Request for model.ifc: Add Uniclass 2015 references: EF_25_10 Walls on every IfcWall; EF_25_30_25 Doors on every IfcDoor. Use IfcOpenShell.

First a look at what the model holds.

```python
import ifcopenshell

model = ifcopenshell.open("model.ifc")
print(model.schema)
print("classifications:", [c.Name for c in model.by_type("IfcClassification")])
for ifc_class in ("IfcDoor", "IfcRoof", "IfcStair", "IfcWall", "IfcWindow"):
    print(ifc_class, len(model.by_type(ifc_class)))
```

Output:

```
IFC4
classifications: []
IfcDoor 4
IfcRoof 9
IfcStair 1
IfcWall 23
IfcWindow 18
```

```python
import ifcopenshell
import ifcopenshell.api.classification

model = ifcopenshell.open("model.ifc")

system = ifcopenshell.api.classification.add_classification(model, classification="Uniclass 2015")

codes = {
    "IfcWall": ("EF_25_10", "Walls"),
    "IfcDoor": ("EF_25_30_25", "Doors"),
}
for ifc_class, (code, name) in codes.items():
    products = model.by_type(ifc_class)
    ifcopenshell.api.classification.add_reference(
        model, products=products, classification=system, identification=code, name=name
    )
    print(code, len(products))

model.write("model_rev.ifc")
```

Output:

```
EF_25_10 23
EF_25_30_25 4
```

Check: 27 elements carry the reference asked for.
